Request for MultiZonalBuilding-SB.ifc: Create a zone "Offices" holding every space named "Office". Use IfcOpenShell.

First a look at what the model holds.

```python
import ifcopenshell

model = ifcopenshell.open("MultiZonalBuilding-SB.ifc")
print(model.schema)
seen = {}
for space in model.by_type("IfcSpace"):
    seen[space.LongName] = seen.get(space.LongName, 0) + 1
for name, count in sorted(seen.items(), key=str):
    print(count, "x", name)
print("zones:", [z.Name for z in model.by_type("IfcZone")][:20])
```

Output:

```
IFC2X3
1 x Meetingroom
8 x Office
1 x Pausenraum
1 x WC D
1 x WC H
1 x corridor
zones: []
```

```python
import ifcopenshell
import ifcopenshell.api.group
import ifcopenshell.api.root

model = ifcopenshell.open("MultiZonalBuilding-SB.ifc")

names = {"Office"}
spaces = [s for s in model.by_type("IfcSpace") if s.LongName in names]

zone = ifcopenshell.api.root.create_entity(model, ifc_class="IfcZone", name="Offices")
ifcopenshell.api.group.assign_group(model, products=spaces, group=zone)
print(len(spaces), "spaces in", zone.Name)

model.write("MultiZonalBuilding-SB_edited.ifc")
```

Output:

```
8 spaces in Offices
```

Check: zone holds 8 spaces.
